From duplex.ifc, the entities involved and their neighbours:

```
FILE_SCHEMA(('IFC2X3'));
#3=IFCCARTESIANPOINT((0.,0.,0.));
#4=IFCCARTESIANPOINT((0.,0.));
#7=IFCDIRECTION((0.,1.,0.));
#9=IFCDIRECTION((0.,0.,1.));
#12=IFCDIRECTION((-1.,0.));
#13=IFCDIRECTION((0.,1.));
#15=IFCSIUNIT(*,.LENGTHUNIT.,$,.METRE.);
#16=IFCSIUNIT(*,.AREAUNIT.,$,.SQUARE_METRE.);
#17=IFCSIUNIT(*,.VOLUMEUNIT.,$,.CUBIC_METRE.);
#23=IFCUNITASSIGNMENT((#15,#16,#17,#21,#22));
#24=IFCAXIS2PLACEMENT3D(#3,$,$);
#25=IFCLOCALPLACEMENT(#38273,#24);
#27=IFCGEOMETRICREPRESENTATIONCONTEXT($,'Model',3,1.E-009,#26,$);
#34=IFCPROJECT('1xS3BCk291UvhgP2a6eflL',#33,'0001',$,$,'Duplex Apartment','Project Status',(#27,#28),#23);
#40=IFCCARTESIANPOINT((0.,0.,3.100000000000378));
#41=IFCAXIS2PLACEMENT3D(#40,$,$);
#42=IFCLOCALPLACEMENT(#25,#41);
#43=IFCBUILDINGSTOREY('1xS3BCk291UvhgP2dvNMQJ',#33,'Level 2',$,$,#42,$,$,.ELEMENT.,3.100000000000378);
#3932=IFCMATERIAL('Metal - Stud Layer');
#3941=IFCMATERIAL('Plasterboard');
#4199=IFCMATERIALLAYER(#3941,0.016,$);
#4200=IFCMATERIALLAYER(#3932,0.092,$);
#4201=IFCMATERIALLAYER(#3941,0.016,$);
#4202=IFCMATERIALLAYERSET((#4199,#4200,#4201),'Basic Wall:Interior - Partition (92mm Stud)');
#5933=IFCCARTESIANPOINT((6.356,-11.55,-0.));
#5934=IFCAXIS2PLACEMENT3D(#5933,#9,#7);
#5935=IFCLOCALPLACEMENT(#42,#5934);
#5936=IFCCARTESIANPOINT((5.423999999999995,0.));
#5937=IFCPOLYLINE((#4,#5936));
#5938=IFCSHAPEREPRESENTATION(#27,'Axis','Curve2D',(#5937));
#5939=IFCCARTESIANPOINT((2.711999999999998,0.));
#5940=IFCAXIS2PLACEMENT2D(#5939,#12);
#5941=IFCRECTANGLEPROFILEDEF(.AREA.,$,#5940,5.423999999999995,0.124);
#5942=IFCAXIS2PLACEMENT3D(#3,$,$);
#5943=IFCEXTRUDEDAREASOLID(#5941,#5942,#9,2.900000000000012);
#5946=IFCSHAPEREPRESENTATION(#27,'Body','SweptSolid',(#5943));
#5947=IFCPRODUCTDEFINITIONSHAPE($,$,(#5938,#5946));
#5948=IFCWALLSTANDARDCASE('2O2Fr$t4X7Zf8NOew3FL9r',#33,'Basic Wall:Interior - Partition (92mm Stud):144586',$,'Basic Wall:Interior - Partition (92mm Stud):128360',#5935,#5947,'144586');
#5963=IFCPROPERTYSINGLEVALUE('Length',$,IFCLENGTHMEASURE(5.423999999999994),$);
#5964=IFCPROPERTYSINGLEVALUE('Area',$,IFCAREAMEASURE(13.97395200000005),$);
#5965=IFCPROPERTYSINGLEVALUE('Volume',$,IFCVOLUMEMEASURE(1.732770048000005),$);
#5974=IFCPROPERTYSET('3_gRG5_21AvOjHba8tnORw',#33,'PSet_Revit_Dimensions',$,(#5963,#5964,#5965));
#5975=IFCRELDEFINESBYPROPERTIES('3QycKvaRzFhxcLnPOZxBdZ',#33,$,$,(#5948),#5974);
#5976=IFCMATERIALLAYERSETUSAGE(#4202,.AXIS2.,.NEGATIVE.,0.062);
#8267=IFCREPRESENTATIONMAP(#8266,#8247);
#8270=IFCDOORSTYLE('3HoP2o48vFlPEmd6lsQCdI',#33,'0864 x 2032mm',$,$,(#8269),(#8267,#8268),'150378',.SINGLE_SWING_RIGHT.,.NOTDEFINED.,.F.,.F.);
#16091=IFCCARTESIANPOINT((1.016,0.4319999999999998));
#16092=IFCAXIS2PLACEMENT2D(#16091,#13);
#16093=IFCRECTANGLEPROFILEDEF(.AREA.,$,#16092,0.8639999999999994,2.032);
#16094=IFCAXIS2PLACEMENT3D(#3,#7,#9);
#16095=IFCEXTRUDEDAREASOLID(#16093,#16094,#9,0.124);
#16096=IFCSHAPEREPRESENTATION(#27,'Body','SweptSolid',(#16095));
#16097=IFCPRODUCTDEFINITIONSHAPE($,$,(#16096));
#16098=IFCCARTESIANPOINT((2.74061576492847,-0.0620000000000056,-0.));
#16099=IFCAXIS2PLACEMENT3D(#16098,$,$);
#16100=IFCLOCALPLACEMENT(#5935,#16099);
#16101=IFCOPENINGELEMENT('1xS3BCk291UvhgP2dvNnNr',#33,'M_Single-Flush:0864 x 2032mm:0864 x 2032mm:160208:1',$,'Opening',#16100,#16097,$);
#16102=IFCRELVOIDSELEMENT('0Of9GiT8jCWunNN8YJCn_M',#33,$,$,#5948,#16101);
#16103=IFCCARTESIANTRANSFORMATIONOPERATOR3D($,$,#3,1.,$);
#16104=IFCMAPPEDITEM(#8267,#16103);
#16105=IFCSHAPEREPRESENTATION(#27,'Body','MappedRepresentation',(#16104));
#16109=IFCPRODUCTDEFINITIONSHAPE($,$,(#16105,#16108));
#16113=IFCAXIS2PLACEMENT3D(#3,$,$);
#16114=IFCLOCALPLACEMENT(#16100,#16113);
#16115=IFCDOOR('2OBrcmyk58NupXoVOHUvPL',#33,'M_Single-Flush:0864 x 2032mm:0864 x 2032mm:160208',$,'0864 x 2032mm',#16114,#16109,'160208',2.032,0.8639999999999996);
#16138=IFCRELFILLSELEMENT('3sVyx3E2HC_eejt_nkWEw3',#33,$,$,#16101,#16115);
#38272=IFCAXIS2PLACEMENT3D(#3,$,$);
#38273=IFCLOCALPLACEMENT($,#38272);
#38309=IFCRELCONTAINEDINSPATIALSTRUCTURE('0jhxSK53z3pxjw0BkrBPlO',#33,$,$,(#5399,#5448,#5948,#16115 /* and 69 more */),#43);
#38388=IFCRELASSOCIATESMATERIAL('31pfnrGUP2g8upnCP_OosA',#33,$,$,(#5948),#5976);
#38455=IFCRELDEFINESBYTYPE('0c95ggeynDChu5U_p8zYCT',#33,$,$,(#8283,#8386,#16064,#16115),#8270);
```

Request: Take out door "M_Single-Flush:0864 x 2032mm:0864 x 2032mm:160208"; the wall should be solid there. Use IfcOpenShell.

```python
import ifcopenshell
import ifcopenshell.api.feature
import ifcopenshell.api.pset
import ifcopenshell.api.root
import ifcopenshell.geom
import ifcopenshell.util.element
import ifcopenshell.util.shape
import ifcopenshell.util.unit

model = ifcopenshell.open("duplex.ifc")
area_scale = ifcopenshell.util.unit.calculate_unit_scale(model, "AREAUNIT")
volume_scale = ifcopenshell.util.unit.calculate_unit_scale(model, "VOLUMEUNIT")
settings = ifcopenshell.geom.settings()


def volume(element):
    """Net volume in cubic metres, openings subtracted."""
    shape = ifcopenshell.geom.create_shape(settings, element)
    return ifcopenshell.util.shape.get_volume(shape.geometry)


door = model.by_id(16115)
opening = door.FillsVoids[0].RelatingOpeningElement
wall = opening.VoidsElements[0].RelatingBuildingElement
before = volume(wall)

ifcopenshell.api.root.remove_product(model, product=door)
ifcopenshell.api.feature.remove_feature(model, feature=opening)

after = volume(wall)
thickness = 0.124  # wall thickness in metres

# Update the wall's stored quantities.
pset = model.by_id(ifcopenshell.util.element.get_pset(wall, "PSet_Revit_Dimensions", should_inherit=False)["id"])
ifcopenshell.api.pset.edit_pset(model, pset=pset, properties={
    "Area": model.create_entity("IfcAreaMeasure", after / thickness / area_scale),
    "Volume": model.create_entity("IfcVolumeMeasure", after / volume_scale),
})

print(f"wall volume {before:.3f} -> {after:.3f} m3")

model.write("duplex_edited.ifc")
```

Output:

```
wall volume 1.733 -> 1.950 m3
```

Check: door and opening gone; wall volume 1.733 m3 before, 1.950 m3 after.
